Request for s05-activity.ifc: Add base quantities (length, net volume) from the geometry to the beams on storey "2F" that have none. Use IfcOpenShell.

First a look at what the model holds.

```python
import ifcopenshell
import ifcopenshell.util.element
import ifcopenshell.util.unit

model = ifcopenshell.open("s05-activity.ifc")
print(model.schema)
for unit_type in ("LENGTHUNIT", "AREAUNIT", "VOLUMEUNIT"):
    print(unit_type, ifcopenshell.util.unit.calculate_unit_scale(model, unit_type))
storey = next(s for s in model.by_type("IfcBuildingStorey") if s.Name == "2F")
beams = [e for e in ifcopenshell.util.element.get_decomposition(storey) if e.is_a("IfcBeam")]
for e in sorted(beams, key=lambda e: e.id()):
    print(e.id(), e.is_a(), e.Name, list(ifcopenshell.util.element.get_psets(e, qtos_only=True)), sep=" | ")
```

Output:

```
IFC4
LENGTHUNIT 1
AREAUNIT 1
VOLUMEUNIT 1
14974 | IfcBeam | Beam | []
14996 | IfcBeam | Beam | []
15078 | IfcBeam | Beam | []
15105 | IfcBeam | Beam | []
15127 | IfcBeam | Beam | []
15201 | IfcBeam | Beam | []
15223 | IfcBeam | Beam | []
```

```python
import ifcopenshell
import ifcopenshell.api.pset
import ifcopenshell.geom
import ifcopenshell.util.element
import ifcopenshell.util.shape
import ifcopenshell.util.unit

model = ifcopenshell.open("s05-activity.ifc")
unit_scale = ifcopenshell.util.unit.calculate_unit_scale(model)
volume_scale = ifcopenshell.util.unit.calculate_unit_scale(model, "VOLUMEUNIT")
settings = ifcopenshell.geom.settings()

storey = next(s for s in model.by_type("IfcBuildingStorey") if s.Name == "2F")
beams = [e for e in ifcopenshell.util.element.get_decomposition(storey) if e.is_a("IfcBeam")]

for e in sorted(beams, key=lambda e: e.id()):
    if ifcopenshell.util.element.get_psets(e, qtos_only=True, should_inherit=False):
        continue
    # Geometry comes back in metres, in the element's own axes.
    shape = ifcopenshell.geom.create_shape(settings, e)
    values = {
        "Length": ifcopenshell.util.shape.get_max_xyz(shape.geometry) / unit_scale,
        "NetVolume": ifcopenshell.util.shape.get_volume(shape.geometry) / volume_scale,
    }
    qto = ifcopenshell.api.pset.add_qto(model, product=e, name="Qto_BeamBaseQuantities")
    ifcopenshell.api.pset.edit_qto(model, qto=qto, properties=values)
    print(e.id(), {k: round(v, 3) for k, v in values.items()})

model.write("s05-activity_updated.ifc")
```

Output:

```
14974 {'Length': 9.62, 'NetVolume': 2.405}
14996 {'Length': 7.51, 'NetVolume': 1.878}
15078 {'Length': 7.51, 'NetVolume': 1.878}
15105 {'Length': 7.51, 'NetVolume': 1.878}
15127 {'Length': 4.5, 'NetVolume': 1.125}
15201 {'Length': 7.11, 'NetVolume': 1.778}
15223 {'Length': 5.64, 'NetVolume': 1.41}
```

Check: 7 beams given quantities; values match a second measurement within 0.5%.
